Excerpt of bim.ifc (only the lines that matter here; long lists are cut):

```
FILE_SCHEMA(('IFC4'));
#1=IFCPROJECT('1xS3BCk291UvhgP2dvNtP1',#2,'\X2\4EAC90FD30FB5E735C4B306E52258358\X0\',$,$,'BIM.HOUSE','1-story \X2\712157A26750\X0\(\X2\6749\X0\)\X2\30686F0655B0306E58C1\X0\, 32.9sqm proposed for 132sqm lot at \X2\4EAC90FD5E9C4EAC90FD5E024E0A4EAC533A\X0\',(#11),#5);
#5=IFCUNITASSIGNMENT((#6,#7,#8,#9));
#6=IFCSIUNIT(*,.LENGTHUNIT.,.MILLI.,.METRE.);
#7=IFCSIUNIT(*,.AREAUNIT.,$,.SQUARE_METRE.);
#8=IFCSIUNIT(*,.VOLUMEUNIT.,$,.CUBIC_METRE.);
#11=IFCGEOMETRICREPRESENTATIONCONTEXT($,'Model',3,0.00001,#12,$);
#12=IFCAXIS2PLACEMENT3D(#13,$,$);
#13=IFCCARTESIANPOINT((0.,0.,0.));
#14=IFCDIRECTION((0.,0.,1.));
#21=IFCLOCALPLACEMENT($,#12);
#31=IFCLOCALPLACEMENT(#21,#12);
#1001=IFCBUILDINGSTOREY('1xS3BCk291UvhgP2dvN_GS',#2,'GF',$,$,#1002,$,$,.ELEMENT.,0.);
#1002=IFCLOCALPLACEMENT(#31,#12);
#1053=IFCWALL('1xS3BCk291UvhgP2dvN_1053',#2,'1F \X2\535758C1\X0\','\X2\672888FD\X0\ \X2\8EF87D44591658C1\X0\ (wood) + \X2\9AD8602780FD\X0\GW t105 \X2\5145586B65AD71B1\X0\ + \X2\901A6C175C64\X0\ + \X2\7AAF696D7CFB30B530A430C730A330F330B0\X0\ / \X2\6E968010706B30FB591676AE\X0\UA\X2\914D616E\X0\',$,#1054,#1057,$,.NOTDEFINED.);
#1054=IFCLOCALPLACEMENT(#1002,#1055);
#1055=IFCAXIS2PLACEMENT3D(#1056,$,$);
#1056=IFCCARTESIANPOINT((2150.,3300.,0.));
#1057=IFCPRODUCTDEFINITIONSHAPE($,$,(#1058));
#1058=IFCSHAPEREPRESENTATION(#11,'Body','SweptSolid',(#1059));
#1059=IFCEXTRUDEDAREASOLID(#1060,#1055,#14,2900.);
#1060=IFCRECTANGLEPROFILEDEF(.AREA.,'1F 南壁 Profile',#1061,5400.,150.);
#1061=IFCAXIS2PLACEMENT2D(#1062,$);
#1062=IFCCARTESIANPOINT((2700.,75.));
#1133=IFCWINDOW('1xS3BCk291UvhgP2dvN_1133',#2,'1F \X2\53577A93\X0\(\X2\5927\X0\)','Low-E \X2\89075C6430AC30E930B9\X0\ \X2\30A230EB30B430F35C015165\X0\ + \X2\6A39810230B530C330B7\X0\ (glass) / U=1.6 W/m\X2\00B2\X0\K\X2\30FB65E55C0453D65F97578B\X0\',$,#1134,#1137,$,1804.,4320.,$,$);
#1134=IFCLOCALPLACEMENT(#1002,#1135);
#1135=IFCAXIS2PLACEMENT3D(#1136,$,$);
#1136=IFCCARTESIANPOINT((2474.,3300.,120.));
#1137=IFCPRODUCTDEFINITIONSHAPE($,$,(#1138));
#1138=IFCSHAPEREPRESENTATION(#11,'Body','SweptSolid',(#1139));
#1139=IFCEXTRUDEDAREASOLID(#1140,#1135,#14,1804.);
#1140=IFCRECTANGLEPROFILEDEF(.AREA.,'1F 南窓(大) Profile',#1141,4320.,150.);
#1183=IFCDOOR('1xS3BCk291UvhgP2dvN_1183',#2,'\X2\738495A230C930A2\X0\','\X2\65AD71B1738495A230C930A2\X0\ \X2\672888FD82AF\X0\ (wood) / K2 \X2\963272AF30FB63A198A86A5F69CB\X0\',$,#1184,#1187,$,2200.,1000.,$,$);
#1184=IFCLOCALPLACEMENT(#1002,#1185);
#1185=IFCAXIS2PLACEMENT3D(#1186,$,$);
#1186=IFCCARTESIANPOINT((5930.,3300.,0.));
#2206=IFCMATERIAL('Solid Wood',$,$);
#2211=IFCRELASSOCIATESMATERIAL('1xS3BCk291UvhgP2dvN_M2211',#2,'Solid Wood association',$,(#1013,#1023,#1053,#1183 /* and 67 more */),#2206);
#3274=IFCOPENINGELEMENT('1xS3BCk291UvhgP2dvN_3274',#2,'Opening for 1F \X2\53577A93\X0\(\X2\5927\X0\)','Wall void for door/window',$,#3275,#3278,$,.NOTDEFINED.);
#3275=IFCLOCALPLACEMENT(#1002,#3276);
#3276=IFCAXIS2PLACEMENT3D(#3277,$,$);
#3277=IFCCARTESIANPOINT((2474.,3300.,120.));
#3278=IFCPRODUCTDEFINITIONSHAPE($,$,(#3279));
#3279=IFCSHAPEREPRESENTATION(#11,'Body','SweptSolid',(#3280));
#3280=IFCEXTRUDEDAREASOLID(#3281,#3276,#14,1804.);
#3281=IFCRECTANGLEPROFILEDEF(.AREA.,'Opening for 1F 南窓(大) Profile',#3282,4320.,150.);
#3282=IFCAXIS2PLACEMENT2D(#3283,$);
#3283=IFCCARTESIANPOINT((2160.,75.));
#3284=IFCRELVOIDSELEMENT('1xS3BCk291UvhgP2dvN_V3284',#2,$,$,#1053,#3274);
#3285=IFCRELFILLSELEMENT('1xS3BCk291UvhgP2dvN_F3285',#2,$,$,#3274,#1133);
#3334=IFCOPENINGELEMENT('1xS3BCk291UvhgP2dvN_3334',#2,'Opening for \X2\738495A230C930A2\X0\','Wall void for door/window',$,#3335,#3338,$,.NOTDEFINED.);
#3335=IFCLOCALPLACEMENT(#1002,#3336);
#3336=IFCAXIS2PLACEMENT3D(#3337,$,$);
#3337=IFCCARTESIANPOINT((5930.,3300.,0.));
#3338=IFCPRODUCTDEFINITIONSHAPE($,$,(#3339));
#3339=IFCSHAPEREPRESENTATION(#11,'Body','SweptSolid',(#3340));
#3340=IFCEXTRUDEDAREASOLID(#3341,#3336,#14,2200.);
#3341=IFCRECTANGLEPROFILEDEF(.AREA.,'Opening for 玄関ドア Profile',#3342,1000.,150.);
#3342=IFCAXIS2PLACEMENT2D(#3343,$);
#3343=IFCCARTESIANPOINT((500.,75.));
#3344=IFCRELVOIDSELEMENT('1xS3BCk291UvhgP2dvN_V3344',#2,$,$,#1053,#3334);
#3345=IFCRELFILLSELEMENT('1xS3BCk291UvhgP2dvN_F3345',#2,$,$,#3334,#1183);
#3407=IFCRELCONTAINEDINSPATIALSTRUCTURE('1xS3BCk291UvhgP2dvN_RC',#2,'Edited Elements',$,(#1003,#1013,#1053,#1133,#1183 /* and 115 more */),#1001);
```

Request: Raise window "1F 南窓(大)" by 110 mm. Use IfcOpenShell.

```python
import numpy as np
import ifcopenshell
import ifcopenshell.api.geometry
import ifcopenshell.util.placement
import ifcopenshell.util.unit

model = ifcopenshell.open("bim.ifc")
unit_scale = ifcopenshell.util.unit.calculate_unit_scale(model)

window = model.by_guid("1xS3BCk291UvhgP2dvN_1133")
opening = window.FillsVoids[0].RelatingOpeningElement
dz = 0.11 / unit_scale

shift = np.array([0.0, 0.0, dz])
# The window is not placed relative to its opening, so move both.
for product in (opening, window):
    matrix = ifcopenshell.util.placement.get_local_placement(product.ObjectPlacement)
    matrix[:3, 3] += shift
    ifcopenshell.api.geometry.edit_object_placement(model, product=product, matrix=matrix, is_si=False)

print(f"moved by {dz * unit_scale:+.3f} m")

model.write("bim_v2.ifc")
```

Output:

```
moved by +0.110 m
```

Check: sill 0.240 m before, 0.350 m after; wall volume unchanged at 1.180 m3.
